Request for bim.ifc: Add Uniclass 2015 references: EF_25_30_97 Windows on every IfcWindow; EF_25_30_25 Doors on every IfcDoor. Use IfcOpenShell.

First a look at what the model holds.

```python
import ifcopenshell

model = ifcopenshell.open("bim.ifc")
print(model.schema)
print("classifications:", [c.Name for c in model.by_type("IfcClassification")])
for ifc_class in ("IfcDoor", "IfcRoof", "IfcStair", "IfcWall", "IfcWindow"):
    print(ifc_class, len(model.by_type(ifc_class)))
```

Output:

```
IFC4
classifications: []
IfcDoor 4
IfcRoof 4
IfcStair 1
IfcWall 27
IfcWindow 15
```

```python
import ifcopenshell
import ifcopenshell.api.classification

model = ifcopenshell.open("bim.ifc")

system = ifcopenshell.api.classification.add_classification(model, classification="Uniclass 2015")

codes = {
    "IfcWindow": ("EF_25_30_97", "Windows"),
    "IfcDoor": ("EF_25_30_25", "Doors"),
}
for ifc_class, (code, name) in codes.items():
    products = model.by_type(ifc_class)
    ifcopenshell.api.classification.add_reference(
        model, products=products, classification=system, identification=code, name=name
    )
    print(code, len(products))

model.write("bim_updated.ifc")
```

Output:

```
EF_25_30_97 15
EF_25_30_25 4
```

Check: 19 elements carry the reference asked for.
